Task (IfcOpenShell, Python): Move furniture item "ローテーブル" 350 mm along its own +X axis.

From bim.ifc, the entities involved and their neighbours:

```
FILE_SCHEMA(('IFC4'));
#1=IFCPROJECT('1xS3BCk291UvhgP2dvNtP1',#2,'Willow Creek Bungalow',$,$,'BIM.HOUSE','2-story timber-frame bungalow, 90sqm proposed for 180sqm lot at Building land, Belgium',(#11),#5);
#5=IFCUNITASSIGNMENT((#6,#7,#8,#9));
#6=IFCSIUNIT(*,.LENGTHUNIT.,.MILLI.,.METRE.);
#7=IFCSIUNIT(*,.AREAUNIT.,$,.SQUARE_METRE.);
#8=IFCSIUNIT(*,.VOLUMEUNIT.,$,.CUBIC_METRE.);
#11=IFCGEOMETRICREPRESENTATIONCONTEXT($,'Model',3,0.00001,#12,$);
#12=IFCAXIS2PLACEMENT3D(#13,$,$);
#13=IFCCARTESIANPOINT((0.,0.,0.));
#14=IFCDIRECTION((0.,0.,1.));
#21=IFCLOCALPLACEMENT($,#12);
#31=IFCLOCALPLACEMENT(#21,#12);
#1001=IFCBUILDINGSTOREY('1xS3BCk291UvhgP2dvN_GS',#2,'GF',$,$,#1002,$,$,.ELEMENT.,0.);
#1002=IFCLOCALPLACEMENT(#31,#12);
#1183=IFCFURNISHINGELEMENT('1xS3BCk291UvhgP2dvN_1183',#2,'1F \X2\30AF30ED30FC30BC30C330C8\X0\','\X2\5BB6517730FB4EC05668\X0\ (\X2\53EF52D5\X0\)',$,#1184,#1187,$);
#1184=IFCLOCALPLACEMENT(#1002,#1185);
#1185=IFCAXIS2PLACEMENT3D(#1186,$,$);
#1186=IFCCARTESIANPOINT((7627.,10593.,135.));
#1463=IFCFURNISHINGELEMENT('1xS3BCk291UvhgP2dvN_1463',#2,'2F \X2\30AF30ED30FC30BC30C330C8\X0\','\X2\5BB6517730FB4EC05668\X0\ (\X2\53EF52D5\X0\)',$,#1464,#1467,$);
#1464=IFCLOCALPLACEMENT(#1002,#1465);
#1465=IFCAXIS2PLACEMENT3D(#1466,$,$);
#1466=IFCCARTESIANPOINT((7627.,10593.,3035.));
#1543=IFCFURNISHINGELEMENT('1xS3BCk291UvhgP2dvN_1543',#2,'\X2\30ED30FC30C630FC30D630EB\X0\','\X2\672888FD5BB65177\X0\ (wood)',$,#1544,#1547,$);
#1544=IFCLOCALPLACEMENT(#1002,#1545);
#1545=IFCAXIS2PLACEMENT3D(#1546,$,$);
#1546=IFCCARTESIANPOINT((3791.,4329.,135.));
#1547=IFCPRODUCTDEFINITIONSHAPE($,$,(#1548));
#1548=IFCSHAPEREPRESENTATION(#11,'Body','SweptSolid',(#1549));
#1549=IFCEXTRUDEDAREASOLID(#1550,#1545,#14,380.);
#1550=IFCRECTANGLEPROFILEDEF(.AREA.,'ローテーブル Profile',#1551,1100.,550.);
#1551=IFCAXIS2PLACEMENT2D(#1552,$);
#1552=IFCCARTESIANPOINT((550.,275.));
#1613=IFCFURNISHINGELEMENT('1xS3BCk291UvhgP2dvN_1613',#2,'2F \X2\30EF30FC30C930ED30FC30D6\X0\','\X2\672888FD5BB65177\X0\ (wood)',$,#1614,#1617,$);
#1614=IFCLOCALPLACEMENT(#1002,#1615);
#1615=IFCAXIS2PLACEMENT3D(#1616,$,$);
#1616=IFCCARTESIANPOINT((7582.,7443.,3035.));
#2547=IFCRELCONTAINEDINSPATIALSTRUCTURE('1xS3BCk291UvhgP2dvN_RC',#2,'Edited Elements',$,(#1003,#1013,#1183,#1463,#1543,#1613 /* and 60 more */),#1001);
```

```python
import ifcopenshell
import ifcopenshell.api.geometry
import ifcopenshell.util.placement
import ifcopenshell.util.unit

model = ifcopenshell.open("bim.ifc")
unit_scale = ifcopenshell.util.unit.calculate_unit_scale(model)

item = model.by_guid("1xS3BCk291UvhgP2dvN_1543")
matrix = ifcopenshell.util.placement.get_local_placement(item.ObjectPlacement)
matrix[:3, 3] += matrix[:3, 0] * 0.35 / unit_scale
ifcopenshell.api.geometry.edit_object_placement(model, product=item, matrix=matrix, is_si=False)

print(ifcopenshell.util.placement.get_local_placement(item.ObjectPlacement).round(3) + 0.0)

model.write("bim_updated.ifc")
```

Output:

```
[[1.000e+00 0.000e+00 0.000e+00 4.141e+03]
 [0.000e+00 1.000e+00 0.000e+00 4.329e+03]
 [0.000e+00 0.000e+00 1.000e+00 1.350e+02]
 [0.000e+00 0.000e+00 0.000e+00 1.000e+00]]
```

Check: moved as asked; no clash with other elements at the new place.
